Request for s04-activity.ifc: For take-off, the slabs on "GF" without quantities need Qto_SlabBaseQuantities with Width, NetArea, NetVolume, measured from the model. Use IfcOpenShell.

First a look at what the model holds.

```python
import ifcopenshell
import ifcopenshell.util.element
import ifcopenshell.util.unit

model = ifcopenshell.open("s04-activity.ifc")
print(model.schema)
for unit_type in ("LENGTHUNIT", "AREAUNIT", "VOLUMEUNIT"):
    print(unit_type, ifcopenshell.util.unit.calculate_unit_scale(model, unit_type))
storey = next(s for s in model.by_type("IfcBuildingStorey") if s.Name == "GF")
slabs = [e for e in ifcopenshell.util.element.get_decomposition(storey) if e.is_a("IfcSlab")]
for e in sorted(slabs, key=lambda e: e.id()):
    print(e.id(), e.is_a(), e.Name, list(ifcopenshell.util.element.get_psets(e, qtos_only=True)), sep=" | ")
```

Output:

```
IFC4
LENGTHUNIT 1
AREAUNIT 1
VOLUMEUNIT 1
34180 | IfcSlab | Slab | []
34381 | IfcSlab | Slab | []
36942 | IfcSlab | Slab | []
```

```python
import ifcopenshell
import ifcopenshell.api.pset
import ifcopenshell.geom
import ifcopenshell.util.element
import ifcopenshell.util.shape
import ifcopenshell.util.unit

model = ifcopenshell.open("s04-activity.ifc")
unit_scale = ifcopenshell.util.unit.calculate_unit_scale(model)
area_scale = ifcopenshell.util.unit.calculate_unit_scale(model, "AREAUNIT")
volume_scale = ifcopenshell.util.unit.calculate_unit_scale(model, "VOLUMEUNIT")
settings = ifcopenshell.geom.settings()

storey = next(s for s in model.by_type("IfcBuildingStorey") if s.Name == "GF")
slabs = [e for e in ifcopenshell.util.element.get_decomposition(storey) if e.is_a("IfcSlab")]

for e in sorted(slabs, key=lambda e: e.id()):
    if ifcopenshell.util.element.get_psets(e, qtos_only=True, should_inherit=False):
        continue
    # Geometry comes back in metres, in the element's own axes.
    shape = ifcopenshell.geom.create_shape(settings, e)
    values = {
        "Width": ifcopenshell.util.shape.get_z(shape.geometry) / unit_scale,
        "NetArea": ifcopenshell.util.shape.get_footprint_area(shape.geometry) / area_scale,
        "NetVolume": ifcopenshell.util.shape.get_volume(shape.geometry) / volume_scale,
    }
    qto = ifcopenshell.api.pset.add_qto(model, product=e, name="Qto_SlabBaseQuantities")
    ifcopenshell.api.pset.edit_qto(model, qto=qto, properties=values)
    print(e.id(), {k: round(v, 3) for k, v in values.items()})

model.write("s04-activity-out.ifc")
```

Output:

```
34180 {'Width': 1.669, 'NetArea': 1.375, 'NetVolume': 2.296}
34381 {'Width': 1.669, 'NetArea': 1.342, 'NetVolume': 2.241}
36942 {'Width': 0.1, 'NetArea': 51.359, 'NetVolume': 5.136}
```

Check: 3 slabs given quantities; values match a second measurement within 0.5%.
